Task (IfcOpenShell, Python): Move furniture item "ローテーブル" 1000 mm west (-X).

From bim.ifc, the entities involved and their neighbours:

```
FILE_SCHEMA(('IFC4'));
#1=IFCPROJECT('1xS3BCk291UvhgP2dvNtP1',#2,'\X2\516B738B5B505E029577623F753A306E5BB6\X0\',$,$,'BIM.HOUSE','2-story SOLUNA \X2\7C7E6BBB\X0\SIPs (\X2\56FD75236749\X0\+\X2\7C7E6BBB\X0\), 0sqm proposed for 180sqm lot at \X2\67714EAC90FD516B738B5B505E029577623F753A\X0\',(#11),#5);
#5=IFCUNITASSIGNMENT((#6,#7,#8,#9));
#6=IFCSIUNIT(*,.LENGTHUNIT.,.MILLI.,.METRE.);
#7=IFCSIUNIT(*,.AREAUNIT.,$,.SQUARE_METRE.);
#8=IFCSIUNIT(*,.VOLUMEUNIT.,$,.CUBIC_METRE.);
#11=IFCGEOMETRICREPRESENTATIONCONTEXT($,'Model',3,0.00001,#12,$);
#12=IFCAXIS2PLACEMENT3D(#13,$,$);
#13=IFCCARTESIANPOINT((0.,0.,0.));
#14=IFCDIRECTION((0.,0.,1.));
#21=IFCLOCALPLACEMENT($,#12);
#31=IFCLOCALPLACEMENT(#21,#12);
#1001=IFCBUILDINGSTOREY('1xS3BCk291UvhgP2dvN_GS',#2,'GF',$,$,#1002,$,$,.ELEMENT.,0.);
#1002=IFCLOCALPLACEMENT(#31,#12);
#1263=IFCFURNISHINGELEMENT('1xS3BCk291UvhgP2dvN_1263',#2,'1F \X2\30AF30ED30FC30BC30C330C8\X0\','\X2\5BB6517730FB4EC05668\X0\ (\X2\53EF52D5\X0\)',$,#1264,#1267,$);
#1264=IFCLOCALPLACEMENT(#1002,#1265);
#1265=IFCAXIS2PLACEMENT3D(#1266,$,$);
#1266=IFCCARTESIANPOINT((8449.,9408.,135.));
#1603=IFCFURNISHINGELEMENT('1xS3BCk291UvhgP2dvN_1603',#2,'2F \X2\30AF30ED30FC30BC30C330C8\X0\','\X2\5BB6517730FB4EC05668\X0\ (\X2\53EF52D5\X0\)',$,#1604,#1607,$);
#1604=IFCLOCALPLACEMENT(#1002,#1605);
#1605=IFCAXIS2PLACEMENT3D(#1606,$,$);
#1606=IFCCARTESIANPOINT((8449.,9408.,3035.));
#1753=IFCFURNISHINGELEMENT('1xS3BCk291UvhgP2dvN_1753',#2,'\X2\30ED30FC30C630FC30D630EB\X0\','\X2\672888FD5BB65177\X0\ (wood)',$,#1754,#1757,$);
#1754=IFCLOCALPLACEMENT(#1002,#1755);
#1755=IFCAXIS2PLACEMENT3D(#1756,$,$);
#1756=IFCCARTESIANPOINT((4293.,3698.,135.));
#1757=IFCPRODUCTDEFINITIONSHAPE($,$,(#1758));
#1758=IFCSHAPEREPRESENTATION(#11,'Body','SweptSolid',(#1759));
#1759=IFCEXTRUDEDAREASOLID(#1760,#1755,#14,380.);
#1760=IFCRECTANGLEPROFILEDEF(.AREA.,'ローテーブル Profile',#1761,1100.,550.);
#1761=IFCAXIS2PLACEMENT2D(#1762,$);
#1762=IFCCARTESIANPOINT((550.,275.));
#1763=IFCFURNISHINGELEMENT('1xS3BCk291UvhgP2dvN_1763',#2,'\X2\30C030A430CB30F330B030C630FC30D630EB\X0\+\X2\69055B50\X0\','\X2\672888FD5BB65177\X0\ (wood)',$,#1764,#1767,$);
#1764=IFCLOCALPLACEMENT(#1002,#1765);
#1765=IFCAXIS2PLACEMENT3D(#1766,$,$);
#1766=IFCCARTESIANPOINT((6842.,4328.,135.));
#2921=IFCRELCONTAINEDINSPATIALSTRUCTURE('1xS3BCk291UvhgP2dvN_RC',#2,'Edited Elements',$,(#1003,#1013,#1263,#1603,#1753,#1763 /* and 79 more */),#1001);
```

```python
import ifcopenshell
import ifcopenshell.api.geometry
import ifcopenshell.util.placement
import ifcopenshell.util.unit

model = ifcopenshell.open("bim.ifc")
unit_scale = ifcopenshell.util.unit.calculate_unit_scale(model)

item = model.by_guid("1xS3BCk291UvhgP2dvN_1753")
matrix = ifcopenshell.util.placement.get_local_placement(item.ObjectPlacement)
matrix[0, 3] -= 1 / unit_scale
ifcopenshell.api.geometry.edit_object_placement(model, product=item, matrix=matrix, is_si=False)

print(ifcopenshell.util.placement.get_local_placement(item.ObjectPlacement).round(3) + 0.0)

model.write("bim-out.ifc")
```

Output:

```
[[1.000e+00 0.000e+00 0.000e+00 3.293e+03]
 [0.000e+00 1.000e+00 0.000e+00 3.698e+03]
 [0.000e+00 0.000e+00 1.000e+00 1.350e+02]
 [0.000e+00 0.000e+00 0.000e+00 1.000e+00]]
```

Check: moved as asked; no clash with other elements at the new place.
